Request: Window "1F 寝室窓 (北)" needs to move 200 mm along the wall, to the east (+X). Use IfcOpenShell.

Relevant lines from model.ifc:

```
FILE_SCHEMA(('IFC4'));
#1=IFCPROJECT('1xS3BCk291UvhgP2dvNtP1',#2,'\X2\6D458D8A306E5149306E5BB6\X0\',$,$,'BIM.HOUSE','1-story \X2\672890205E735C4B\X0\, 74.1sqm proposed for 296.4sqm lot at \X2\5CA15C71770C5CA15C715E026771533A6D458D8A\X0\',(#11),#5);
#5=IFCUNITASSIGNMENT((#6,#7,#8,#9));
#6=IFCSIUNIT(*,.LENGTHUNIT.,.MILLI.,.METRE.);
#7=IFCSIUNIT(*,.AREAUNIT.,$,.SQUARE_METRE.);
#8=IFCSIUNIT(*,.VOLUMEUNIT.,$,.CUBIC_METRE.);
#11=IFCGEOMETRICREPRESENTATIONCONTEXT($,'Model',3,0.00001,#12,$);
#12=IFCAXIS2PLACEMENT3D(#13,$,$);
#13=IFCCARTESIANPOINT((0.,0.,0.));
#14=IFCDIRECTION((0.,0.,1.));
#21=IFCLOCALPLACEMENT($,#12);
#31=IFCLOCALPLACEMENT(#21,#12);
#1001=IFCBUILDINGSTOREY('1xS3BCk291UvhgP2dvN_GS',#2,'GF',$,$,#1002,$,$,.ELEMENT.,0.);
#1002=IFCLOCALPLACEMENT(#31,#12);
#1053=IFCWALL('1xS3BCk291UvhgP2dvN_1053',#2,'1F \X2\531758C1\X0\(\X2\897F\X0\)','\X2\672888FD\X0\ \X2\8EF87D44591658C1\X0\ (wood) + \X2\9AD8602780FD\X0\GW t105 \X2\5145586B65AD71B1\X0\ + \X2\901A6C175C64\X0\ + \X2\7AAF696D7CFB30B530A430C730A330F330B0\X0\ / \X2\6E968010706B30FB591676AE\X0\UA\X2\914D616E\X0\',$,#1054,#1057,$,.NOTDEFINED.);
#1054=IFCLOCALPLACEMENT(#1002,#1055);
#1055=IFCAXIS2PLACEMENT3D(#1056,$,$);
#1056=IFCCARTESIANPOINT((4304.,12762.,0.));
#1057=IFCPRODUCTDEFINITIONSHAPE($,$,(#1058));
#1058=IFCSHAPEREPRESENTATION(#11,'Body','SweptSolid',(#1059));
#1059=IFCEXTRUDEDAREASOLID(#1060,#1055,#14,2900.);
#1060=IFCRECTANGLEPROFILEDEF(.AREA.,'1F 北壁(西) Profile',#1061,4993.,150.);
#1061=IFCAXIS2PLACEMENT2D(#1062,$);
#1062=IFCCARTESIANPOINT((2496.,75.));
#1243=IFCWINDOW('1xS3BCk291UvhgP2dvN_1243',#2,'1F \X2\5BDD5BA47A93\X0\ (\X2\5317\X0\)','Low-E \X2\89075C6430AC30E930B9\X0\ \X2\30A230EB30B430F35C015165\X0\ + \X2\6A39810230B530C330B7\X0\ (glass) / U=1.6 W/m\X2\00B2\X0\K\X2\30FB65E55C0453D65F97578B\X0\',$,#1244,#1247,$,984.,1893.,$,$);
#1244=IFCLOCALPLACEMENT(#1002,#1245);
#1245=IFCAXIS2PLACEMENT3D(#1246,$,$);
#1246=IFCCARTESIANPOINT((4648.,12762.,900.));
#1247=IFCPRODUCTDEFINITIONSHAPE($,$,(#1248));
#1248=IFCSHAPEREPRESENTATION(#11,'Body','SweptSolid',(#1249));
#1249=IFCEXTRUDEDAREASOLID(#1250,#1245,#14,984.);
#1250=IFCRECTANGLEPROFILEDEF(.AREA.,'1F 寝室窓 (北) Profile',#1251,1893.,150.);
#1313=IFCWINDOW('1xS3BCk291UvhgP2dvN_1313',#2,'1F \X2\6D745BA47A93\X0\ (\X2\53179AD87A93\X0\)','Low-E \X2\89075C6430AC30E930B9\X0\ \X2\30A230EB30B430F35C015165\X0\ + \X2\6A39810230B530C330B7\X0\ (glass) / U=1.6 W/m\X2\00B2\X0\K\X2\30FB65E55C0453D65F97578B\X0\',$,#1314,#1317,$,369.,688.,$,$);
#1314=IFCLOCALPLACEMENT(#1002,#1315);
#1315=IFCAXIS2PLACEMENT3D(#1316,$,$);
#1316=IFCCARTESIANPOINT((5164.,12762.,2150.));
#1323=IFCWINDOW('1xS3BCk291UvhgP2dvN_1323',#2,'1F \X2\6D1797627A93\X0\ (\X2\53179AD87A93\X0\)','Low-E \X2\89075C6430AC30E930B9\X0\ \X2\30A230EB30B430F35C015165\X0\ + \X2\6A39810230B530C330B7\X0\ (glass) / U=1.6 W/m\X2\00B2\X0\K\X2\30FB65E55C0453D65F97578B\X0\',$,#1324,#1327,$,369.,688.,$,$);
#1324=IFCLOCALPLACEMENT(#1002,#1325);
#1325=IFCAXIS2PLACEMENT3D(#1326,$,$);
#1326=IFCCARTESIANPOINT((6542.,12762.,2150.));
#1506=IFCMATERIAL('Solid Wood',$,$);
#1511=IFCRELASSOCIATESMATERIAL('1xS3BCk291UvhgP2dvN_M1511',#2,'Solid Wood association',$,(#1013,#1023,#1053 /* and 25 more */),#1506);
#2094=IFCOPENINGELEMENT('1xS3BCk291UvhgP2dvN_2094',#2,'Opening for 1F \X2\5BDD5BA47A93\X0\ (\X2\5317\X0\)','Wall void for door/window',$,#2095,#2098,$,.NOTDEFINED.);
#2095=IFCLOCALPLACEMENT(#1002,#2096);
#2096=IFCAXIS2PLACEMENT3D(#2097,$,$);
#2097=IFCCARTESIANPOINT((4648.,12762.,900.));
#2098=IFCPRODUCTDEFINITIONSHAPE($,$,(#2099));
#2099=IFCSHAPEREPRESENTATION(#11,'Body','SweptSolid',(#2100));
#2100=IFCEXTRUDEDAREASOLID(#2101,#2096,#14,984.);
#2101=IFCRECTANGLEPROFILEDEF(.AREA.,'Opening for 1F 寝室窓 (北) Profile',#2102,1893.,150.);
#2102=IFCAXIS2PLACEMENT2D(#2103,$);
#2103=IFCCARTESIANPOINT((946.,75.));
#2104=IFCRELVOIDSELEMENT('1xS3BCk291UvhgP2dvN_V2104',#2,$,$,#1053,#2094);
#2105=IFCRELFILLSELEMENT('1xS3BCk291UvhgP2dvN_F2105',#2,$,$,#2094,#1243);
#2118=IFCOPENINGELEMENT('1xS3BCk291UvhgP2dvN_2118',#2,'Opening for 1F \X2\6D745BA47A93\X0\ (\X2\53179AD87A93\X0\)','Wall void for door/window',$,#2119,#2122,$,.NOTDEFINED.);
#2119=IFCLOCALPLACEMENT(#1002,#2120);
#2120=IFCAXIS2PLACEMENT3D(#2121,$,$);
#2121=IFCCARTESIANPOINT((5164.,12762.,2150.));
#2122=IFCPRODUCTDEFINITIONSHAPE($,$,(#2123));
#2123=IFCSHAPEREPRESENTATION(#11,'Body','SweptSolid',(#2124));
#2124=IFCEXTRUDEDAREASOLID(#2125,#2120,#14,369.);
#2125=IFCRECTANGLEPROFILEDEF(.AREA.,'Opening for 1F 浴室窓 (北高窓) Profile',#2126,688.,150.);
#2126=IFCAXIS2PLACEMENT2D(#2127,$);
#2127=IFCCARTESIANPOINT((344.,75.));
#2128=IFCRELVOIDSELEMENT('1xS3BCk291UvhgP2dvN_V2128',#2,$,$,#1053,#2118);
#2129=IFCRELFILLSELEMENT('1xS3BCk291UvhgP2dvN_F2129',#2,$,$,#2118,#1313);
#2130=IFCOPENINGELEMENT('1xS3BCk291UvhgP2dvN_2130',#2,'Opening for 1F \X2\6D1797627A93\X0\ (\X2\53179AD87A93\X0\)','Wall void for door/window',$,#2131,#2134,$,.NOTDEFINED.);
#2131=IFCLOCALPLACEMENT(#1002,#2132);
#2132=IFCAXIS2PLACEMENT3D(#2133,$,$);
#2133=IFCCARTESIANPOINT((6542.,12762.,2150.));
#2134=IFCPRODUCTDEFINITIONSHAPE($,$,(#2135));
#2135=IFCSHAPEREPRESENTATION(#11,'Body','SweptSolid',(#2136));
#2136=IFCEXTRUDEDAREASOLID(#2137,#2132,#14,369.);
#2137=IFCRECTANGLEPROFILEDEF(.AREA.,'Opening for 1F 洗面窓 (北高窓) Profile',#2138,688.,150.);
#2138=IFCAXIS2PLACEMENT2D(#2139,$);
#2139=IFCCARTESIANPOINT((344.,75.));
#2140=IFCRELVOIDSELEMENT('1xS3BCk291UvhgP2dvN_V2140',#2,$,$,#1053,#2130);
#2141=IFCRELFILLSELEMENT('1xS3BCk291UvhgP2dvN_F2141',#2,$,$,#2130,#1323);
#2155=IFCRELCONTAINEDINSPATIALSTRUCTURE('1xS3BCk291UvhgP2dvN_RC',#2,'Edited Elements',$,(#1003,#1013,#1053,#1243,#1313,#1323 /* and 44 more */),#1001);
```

```python
import ifcopenshell
import ifcopenshell.api.geometry
import ifcopenshell.util.placement
import ifcopenshell.util.unit

model = ifcopenshell.open("model.ifc")
unit_scale = ifcopenshell.util.unit.calculate_unit_scale(model)

window = model.by_guid("1xS3BCk291UvhgP2dvN_1243")
opening = window.FillsVoids[0].RelatingOpeningElement
wall = opening.VoidsElements[0].RelatingBuildingElement

wall_matrix = ifcopenshell.util.placement.get_local_placement(wall.ObjectPlacement)
shift = wall_matrix[:3, 0] * 0.2 / unit_scale
before = ifcopenshell.util.placement.get_local_placement(window.ObjectPlacement)[:3, 3].copy()

# The window is not placed relative to its opening, so move both.
for product in (opening, window):
    matrix = ifcopenshell.util.placement.get_local_placement(product.ObjectPlacement)
    matrix[:3, 3] += shift
    ifcopenshell.api.geometry.edit_object_placement(model, product=product, matrix=matrix, is_si=False)

after = ifcopenshell.util.placement.get_local_placement(window.ObjectPlacement)[:3, 3]
print("window moved by", (after - before).round(3) + 0.0)

model.write("model_edited.ifc")
```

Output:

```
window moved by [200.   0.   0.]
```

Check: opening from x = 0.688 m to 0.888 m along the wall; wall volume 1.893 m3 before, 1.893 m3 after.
